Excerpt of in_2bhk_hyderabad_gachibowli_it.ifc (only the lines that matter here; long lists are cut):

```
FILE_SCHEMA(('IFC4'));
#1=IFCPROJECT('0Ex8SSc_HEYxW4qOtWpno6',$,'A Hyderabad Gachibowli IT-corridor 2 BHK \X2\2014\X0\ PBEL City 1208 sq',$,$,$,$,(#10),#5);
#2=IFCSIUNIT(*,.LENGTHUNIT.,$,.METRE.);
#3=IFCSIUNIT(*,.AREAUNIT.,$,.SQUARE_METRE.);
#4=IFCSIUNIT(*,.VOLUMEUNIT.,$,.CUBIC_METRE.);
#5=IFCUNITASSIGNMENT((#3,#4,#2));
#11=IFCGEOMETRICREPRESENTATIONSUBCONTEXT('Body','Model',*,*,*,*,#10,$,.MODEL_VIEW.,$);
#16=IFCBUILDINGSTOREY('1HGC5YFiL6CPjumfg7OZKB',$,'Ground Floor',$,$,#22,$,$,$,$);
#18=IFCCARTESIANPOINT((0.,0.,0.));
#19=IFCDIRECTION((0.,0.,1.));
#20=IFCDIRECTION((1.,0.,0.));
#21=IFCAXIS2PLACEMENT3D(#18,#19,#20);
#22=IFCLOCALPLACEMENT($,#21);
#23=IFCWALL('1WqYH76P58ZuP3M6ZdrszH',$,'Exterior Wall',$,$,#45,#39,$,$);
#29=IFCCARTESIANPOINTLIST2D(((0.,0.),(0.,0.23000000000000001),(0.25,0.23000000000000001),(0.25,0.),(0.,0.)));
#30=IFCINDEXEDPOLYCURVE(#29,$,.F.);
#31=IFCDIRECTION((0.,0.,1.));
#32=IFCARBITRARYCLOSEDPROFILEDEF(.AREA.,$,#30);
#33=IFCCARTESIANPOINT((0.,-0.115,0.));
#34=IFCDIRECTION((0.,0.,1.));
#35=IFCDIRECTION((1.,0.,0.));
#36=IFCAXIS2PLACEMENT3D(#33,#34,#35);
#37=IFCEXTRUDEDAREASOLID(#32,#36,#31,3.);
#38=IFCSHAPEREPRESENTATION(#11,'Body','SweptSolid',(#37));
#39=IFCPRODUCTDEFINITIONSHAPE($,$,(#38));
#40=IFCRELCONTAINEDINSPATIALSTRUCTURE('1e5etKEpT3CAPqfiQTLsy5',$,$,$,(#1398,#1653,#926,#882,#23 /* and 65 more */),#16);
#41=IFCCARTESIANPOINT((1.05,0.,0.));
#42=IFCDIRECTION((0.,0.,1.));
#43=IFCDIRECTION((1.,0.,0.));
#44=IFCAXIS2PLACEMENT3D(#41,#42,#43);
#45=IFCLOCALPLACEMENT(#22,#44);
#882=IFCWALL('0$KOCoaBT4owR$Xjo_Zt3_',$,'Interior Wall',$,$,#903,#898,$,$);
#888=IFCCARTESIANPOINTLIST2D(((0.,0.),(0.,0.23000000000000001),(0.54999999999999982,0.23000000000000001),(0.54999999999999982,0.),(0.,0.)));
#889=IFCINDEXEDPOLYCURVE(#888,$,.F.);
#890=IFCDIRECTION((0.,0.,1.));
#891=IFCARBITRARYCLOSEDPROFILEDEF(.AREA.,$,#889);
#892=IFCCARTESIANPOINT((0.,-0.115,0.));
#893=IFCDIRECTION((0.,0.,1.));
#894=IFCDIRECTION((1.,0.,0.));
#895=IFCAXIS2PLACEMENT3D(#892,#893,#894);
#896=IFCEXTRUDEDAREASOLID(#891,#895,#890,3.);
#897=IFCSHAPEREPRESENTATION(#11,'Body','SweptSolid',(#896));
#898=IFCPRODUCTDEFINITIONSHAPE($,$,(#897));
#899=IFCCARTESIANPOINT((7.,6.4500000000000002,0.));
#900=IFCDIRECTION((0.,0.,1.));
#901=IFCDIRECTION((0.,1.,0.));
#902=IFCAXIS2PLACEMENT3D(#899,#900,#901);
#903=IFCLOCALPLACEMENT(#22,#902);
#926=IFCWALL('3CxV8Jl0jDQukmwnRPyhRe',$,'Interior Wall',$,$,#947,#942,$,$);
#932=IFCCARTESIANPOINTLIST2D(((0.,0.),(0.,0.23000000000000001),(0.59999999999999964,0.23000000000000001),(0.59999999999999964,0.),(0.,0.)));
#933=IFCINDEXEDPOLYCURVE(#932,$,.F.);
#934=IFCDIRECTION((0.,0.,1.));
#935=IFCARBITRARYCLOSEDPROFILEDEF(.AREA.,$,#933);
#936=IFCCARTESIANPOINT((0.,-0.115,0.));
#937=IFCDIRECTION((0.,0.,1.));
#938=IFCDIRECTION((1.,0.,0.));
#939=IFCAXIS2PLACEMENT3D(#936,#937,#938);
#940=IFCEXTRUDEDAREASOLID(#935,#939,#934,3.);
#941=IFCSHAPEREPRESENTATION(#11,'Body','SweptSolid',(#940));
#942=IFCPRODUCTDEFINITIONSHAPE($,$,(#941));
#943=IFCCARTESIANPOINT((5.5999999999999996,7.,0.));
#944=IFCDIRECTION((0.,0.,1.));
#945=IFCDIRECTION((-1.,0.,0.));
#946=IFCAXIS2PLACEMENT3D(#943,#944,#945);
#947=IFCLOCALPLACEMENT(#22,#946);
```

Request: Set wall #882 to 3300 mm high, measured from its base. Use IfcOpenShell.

```python
import ifcopenshell
import ifcopenshell.geom
import ifcopenshell.util.representation
import ifcopenshell.util.shape
import ifcopenshell.util.unit

model = ifcopenshell.open("in_2bhk_hyderabad_gachibowli_it.ifc")
unit_scale = ifcopenshell.util.unit.calculate_unit_scale(model)
settings = ifcopenshell.geom.settings()


def volume(element):
    """Net volume in cubic metres, openings subtracted."""
    shape = ifcopenshell.geom.create_shape(settings, element)
    return ifcopenshell.util.shape.get_volume(shape.geometry)


wall = model.by_guid("0$KOCoaBT4owR$Xjo_Zt3_")
before = volume(wall)

body = ifcopenshell.util.representation.get_representation(wall, "Model", "Body")
solid = body.Items[0]
old_height = solid.Depth
solid.Depth = 3.3 / unit_scale
after = volume(wall)

print(f"height {old_height:g} -> {solid.Depth:g}, volume {before:.3f} -> {after:.3f} m3")

model.write("in_2bhk_hyderabad_gachibowli_it_rev.ifc")
```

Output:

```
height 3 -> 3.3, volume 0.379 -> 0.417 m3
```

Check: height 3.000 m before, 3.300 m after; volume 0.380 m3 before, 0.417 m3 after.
